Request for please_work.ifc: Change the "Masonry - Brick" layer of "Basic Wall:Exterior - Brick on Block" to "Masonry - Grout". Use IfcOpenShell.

First a look at what the model holds.

```python
import ifcopenshell
import ifcopenshell.util.element

model = ifcopenshell.open("please_work.ifc")
print(model.schema)
for layer_set in model.by_type("IfcMaterialLayerSet"):
    if layer_set.LayerSetName == "Basic Wall:Exterior - Brick on Block":
        for layer in layer_set.MaterialLayers:
            print(layer.id(), layer.Material and layer.Material.Name, layer.LayerThickness, sep=" | ")
        print(len(ifcopenshell.util.element.get_elements_by_material(model, layer_set)), "elements and types use it")
print(sorted(m.Name for m in model.by_type("IfcMaterial") if m.Name)[:60])
```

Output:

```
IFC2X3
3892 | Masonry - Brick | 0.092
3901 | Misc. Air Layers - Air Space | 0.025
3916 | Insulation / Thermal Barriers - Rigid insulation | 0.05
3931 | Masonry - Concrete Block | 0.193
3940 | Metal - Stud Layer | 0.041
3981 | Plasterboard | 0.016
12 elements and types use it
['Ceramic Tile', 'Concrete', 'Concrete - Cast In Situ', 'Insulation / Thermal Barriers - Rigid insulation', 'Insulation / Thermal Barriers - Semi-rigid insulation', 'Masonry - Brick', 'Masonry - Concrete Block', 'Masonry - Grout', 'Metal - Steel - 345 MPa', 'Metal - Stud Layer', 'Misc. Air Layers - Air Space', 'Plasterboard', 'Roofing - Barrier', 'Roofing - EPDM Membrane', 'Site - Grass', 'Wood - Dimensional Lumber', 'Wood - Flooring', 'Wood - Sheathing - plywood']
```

```python
import ifcopenshell
import ifcopenshell.api.material

model = ifcopenshell.open("please_work.ifc")

layer_set = next(s for s in model.by_type("IfcMaterialLayerSet") if s.LayerSetName == "Basic Wall:Exterior - Brick on Block")
layer = next(l for l in layer_set.MaterialLayers if l.Material and l.Material.Name == "Masonry - Brick")
material = next(m for m in model.by_type("IfcMaterial") if m.Name == "Masonry - Grout")

# Point this one layer at the other material; renaming the old one would change it everywhere.
ifcopenshell.api.material.edit_layer(model, layer=layer, attributes={}, material=material)

print([l.Material.Name if l.Material else None for l in layer_set.MaterialLayers])

model.write("please_work-out.ifc")
```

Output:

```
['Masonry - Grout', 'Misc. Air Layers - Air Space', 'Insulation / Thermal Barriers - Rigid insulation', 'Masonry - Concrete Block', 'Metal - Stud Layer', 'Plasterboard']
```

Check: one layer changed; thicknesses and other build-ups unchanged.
